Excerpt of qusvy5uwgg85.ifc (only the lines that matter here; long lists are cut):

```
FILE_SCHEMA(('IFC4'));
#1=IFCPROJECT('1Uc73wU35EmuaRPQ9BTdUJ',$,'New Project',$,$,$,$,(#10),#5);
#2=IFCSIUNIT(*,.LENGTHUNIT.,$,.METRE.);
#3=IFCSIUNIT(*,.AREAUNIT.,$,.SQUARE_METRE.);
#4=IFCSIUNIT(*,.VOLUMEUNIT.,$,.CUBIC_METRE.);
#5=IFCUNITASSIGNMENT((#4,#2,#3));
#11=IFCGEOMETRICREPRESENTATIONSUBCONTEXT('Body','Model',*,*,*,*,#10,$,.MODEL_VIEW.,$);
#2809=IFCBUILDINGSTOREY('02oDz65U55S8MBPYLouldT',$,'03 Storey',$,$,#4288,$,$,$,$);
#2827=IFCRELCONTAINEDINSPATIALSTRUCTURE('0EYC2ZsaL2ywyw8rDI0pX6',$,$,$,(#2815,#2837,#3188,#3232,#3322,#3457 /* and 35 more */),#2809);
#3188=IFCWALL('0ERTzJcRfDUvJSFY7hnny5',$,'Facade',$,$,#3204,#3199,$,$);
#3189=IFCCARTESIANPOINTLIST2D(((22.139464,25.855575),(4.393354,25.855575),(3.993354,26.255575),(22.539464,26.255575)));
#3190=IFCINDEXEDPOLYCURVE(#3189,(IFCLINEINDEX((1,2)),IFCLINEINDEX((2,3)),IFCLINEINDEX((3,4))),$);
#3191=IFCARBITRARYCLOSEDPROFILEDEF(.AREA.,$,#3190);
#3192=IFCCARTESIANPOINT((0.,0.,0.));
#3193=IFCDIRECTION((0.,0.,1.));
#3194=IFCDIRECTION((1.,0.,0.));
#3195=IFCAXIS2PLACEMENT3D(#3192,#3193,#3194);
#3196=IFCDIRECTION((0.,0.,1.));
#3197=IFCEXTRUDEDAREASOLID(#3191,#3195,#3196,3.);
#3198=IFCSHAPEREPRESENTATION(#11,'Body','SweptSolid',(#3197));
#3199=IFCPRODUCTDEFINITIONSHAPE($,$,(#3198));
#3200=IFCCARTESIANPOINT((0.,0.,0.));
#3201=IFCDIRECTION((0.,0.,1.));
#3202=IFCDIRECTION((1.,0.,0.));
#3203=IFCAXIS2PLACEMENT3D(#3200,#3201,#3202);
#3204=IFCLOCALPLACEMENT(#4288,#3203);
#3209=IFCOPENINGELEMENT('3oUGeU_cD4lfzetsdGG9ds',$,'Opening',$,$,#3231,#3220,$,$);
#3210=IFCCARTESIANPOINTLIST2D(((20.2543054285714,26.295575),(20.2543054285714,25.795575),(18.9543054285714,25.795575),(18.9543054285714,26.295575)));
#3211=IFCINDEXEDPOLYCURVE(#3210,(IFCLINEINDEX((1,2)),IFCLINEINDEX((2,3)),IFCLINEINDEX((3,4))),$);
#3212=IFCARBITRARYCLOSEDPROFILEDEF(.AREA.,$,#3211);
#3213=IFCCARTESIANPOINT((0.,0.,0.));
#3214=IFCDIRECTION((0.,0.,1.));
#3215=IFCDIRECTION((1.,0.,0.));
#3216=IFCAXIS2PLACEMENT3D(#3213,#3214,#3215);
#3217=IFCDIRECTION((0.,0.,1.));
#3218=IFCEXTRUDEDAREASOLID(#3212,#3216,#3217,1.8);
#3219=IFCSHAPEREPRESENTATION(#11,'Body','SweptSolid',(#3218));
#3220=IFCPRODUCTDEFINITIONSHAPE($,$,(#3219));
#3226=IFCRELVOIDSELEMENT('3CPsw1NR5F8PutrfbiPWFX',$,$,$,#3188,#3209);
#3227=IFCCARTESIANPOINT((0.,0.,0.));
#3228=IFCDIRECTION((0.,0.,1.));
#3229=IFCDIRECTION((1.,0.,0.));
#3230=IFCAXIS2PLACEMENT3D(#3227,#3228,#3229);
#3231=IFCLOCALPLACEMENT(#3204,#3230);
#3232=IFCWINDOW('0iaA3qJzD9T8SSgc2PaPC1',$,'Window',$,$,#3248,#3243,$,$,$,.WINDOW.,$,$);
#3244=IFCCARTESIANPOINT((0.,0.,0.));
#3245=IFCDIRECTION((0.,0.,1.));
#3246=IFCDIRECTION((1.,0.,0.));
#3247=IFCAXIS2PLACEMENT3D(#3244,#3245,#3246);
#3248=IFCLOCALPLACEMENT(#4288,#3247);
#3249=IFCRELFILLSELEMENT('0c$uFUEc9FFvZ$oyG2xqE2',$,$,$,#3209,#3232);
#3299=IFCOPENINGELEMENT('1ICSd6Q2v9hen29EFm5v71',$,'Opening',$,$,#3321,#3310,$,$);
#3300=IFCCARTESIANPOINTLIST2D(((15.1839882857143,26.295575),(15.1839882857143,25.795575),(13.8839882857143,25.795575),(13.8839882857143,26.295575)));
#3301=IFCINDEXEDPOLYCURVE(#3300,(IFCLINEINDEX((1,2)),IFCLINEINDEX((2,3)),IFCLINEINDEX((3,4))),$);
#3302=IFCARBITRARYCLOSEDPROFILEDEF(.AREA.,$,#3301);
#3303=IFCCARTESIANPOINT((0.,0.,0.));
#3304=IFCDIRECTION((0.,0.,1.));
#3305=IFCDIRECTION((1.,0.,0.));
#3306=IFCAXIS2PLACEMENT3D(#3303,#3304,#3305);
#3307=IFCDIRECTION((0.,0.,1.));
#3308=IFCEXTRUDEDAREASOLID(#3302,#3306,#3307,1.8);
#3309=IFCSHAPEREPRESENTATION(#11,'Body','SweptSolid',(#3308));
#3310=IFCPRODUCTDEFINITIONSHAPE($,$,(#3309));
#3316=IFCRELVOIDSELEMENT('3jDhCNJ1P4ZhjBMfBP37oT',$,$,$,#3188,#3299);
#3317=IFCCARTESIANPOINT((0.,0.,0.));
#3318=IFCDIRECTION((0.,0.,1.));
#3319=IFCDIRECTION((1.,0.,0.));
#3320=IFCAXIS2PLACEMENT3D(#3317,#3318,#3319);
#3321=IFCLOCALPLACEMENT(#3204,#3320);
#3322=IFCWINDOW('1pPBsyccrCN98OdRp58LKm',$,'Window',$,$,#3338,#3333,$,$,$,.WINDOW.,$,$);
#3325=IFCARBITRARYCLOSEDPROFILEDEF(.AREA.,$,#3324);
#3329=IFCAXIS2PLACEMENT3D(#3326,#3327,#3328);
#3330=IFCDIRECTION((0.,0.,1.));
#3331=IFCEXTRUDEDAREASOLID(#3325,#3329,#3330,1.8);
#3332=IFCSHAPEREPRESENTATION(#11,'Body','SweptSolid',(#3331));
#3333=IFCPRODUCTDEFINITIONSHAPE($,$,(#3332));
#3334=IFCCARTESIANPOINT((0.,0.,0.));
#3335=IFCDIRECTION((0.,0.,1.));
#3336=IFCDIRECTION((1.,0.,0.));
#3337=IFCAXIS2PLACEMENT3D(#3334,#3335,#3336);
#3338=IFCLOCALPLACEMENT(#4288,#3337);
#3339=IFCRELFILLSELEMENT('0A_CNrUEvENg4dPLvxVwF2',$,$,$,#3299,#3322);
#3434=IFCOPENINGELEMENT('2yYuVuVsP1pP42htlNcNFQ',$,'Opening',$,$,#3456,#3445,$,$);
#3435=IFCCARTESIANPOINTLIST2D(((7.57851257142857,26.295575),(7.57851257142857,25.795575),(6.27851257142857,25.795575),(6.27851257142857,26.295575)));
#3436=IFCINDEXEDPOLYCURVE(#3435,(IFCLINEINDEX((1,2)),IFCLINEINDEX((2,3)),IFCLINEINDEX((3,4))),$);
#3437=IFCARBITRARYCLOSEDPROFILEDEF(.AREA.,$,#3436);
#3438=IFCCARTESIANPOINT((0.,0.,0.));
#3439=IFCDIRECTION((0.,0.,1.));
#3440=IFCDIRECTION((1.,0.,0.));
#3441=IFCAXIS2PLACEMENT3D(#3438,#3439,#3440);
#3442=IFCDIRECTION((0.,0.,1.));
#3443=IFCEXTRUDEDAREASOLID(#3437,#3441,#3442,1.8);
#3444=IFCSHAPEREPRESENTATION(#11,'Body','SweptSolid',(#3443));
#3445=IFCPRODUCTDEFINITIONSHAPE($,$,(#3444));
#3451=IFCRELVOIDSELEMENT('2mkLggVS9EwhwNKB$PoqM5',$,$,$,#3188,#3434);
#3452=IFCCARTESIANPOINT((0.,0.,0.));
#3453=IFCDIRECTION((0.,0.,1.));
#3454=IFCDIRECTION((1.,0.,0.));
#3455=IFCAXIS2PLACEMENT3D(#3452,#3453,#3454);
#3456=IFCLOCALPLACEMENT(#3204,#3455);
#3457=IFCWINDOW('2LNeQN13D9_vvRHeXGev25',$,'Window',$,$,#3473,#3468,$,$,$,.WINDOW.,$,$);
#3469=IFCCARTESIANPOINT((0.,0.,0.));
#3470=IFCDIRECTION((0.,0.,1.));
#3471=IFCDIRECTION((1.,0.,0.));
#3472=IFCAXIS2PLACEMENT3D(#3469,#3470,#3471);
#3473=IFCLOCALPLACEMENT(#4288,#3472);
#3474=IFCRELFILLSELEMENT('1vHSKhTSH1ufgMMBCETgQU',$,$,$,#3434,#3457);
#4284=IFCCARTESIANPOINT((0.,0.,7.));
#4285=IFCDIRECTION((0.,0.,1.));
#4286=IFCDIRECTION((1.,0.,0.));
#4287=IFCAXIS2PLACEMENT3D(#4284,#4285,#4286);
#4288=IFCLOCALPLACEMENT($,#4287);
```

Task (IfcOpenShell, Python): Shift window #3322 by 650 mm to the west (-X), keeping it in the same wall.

```python
import ifcopenshell
import ifcopenshell.api.geometry
import ifcopenshell.util.placement

model = ifcopenshell.open("qusvy5uwgg85.ifc")

window = model.by_guid("1pPBsyccrCN98OdRp58LKm")
opening = window.FillsVoids[0].RelatingOpeningElement
wall = opening.VoidsElements[0].RelatingBuildingElement

wall_matrix = ifcopenshell.util.placement.get_local_placement(wall.ObjectPlacement)
shift = wall_matrix[:3, 0] * -0.65
before = ifcopenshell.util.placement.get_local_placement(window.ObjectPlacement)[:3, 3].copy()

# The window is not placed relative to its opening, so move both.
for product in (opening, window):
    matrix = ifcopenshell.util.placement.get_local_placement(product.ObjectPlacement)
    matrix[:3, 3] += shift
    ifcopenshell.api.geometry.edit_object_placement(model, product=product, matrix=matrix, is_si=False)

after = ifcopenshell.util.placement.get_local_placement(window.ObjectPlacement)[:3, 3]
print("window moved by", (after - before).round(3) + 0.0)

model.write("qusvy5uwgg85_v2.ifc")
```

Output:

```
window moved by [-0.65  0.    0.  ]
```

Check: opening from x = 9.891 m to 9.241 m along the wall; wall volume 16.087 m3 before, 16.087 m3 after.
